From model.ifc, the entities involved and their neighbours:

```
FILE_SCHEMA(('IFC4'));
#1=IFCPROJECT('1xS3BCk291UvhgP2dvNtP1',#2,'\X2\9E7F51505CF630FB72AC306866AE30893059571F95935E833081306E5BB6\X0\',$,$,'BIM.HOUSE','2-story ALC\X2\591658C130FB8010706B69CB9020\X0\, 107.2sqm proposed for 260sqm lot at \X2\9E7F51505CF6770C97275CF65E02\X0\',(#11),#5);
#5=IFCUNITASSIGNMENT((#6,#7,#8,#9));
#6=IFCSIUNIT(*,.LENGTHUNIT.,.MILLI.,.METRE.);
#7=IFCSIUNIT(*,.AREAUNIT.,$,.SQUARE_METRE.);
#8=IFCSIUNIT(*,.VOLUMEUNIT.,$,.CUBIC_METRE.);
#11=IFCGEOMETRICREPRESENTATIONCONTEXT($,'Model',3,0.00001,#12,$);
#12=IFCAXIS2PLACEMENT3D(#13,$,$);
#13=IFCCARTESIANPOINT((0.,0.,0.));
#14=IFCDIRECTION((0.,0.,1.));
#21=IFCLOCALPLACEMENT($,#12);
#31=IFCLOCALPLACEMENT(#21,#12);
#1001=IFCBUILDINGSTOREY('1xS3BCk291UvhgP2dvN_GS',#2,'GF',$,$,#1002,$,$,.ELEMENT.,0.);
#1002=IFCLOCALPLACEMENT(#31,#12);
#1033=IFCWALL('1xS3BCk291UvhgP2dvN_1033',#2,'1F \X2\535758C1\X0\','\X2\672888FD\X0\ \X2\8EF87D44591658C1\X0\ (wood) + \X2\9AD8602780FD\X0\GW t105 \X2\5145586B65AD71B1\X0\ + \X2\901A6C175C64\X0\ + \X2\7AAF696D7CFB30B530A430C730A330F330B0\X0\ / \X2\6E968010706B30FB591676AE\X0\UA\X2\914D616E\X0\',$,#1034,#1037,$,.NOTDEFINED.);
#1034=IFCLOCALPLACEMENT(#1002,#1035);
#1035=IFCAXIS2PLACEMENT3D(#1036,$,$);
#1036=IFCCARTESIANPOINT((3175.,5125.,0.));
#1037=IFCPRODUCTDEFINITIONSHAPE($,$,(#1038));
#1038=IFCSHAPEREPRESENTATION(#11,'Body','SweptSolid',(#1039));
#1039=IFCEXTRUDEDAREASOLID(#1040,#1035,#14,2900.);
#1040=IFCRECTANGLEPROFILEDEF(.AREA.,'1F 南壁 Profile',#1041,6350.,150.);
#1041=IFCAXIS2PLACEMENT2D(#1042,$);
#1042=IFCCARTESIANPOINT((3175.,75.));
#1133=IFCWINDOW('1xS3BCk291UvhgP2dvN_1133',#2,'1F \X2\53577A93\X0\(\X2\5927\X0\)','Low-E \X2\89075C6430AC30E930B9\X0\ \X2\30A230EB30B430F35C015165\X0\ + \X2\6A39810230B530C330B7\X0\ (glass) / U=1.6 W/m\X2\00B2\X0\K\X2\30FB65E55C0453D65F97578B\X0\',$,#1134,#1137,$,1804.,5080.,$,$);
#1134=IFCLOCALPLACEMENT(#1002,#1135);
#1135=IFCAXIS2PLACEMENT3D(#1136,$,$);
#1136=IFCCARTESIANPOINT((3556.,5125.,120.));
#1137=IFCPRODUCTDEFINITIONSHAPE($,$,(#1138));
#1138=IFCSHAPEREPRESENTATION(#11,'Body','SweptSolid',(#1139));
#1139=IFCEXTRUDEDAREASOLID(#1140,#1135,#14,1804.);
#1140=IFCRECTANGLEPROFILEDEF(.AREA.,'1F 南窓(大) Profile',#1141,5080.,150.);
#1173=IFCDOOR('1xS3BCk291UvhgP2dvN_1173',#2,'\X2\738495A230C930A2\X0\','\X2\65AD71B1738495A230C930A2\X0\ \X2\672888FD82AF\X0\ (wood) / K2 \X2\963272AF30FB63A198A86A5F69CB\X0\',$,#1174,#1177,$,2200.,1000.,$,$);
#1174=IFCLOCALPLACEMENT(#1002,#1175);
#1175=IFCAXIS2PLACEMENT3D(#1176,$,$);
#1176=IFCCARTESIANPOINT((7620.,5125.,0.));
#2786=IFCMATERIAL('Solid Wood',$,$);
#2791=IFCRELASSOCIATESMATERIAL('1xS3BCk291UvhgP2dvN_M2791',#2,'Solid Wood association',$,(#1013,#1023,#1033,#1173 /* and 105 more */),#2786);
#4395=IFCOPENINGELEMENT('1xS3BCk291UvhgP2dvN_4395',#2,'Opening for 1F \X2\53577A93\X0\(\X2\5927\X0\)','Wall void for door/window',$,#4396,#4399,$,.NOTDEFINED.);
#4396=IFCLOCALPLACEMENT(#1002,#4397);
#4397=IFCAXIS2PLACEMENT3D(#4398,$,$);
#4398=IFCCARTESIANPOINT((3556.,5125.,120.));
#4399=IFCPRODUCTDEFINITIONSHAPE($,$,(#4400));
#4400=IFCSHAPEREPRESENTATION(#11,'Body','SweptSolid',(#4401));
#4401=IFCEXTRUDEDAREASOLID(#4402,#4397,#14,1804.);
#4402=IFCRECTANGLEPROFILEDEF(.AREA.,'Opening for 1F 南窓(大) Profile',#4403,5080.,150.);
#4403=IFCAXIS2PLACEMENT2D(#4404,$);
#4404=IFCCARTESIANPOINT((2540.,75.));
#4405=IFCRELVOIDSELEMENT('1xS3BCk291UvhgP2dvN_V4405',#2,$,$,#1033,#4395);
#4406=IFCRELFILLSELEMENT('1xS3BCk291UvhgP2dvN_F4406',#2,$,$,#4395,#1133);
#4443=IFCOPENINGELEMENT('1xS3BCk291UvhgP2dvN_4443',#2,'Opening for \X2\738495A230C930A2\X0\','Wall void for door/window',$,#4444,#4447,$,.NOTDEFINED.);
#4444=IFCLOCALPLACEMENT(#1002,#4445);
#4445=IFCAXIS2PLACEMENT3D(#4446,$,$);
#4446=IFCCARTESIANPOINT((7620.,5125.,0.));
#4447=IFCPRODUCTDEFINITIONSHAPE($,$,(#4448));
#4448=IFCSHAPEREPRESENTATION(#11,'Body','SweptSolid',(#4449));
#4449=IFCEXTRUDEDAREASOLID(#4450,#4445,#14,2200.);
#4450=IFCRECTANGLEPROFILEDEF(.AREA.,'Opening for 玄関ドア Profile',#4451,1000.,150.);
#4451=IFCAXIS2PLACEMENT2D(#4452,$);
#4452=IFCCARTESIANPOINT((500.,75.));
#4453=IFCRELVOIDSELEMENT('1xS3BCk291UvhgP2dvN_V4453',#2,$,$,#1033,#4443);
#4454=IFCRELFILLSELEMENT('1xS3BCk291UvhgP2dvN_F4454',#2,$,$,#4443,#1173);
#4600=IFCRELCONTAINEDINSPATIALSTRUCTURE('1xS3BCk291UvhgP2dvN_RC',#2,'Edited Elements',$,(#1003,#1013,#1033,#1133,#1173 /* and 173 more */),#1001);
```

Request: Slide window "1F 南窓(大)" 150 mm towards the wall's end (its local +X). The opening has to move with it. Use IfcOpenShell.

```python
import ifcopenshell
import ifcopenshell.api.geometry
import ifcopenshell.util.placement
import ifcopenshell.util.unit

model = ifcopenshell.open("model.ifc")
unit_scale = ifcopenshell.util.unit.calculate_unit_scale(model)

window = model.by_guid("1xS3BCk291UvhgP2dvN_1133")
opening = window.FillsVoids[0].RelatingOpeningElement
wall = opening.VoidsElements[0].RelatingBuildingElement

wall_matrix = ifcopenshell.util.placement.get_local_placement(wall.ObjectPlacement)
shift = wall_matrix[:3, 0] * 0.15 / unit_scale
before = ifcopenshell.util.placement.get_local_placement(window.ObjectPlacement)[:3, 3].copy()

# The window is not placed relative to its opening, so move both.
for product in (opening, window):
    matrix = ifcopenshell.util.placement.get_local_placement(product.ObjectPlacement)
    matrix[:3, 3] += shift
    ifcopenshell.api.geometry.edit_object_placement(model, product=product, matrix=matrix, is_si=False)

after = ifcopenshell.util.placement.get_local_placement(window.ObjectPlacement)[:3, 3]
print("window moved by", (after - before).round(3) + 0.0)

model.write("model_edited.ifc")
```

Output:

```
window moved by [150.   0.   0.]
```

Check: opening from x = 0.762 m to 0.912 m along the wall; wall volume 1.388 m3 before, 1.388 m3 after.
